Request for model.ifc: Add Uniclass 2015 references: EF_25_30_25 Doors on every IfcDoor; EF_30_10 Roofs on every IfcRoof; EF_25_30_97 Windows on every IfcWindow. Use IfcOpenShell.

First a look at what the model holds.

```python
import ifcopenshell

model = ifcopenshell.open("model.ifc")
print(model.schema)
print("classifications:", [c.Name for c in model.by_type("IfcClassification")])
for ifc_class in ("IfcDoor", "IfcRoof", "IfcStair", "IfcWall", "IfcWindow"):
    print(ifc_class, len(model.by_type(ifc_class)))
```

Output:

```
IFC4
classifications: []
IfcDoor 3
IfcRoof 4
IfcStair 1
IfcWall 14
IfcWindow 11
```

```python
import ifcopenshell
import ifcopenshell.api.classification

model = ifcopenshell.open("model.ifc")

system = ifcopenshell.api.classification.add_classification(model, classification="Uniclass 2015")

codes = {
    "IfcDoor": ("EF_25_30_25", "Doors"),
    "IfcRoof": ("EF_30_10", "Roofs"),
    "IfcWindow": ("EF_25_30_97", "Windows"),
}
for ifc_class, (code, name) in codes.items():
    products = model.by_type(ifc_class)
    ifcopenshell.api.classification.add_reference(
        model, products=products, classification=system, identification=code, name=name
    )
    print(code, len(products))

model.write("model_updated.ifc")
```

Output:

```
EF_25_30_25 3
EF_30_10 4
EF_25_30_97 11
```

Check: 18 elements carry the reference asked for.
